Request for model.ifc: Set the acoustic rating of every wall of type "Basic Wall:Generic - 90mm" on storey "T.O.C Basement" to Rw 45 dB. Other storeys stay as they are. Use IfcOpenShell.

First a look at what the model holds.

```python
import ifcopenshell
import ifcopenshell.util.element

model = ifcopenshell.open("model.ifc")
print(model.schema)
storey = next(s for s in model.by_type("IfcBuildingStorey") if s.Name == "T.O.C Basement")
walls = [e for e in ifcopenshell.util.element.get_decomposition(storey) if e.is_a("IfcWall")]
seen = {}
for e in walls:
    element_type = ifcopenshell.util.element.get_type(e)
    key = (element_type.Name if element_type != e and element_type else None, ifcopenshell.util.element.get_pset(e, "Pset_WallCommon", "AcousticRating"))
    seen[key] = seen.get(key, 0) + 1
for (name, value), count in sorted(seen.items(), key=str):
    print(count, "x", name, "|", value)
```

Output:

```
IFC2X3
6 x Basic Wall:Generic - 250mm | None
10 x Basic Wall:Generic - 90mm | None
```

```python
import ifcopenshell
import ifcopenshell.api.pset
import ifcopenshell.util.element

model = ifcopenshell.open("model.ifc")

storey = next(s for s in model.by_type("IfcBuildingStorey") if s.Name == "T.O.C Basement")
walls = [e for e in ifcopenshell.util.element.get_decomposition(storey) if e.is_a("IfcWall")]

count = 0
for e in walls:
    element_type = ifcopenshell.util.element.get_type(e)
    if element_type in (None, e) or element_type.Name != "Basic Wall:Generic - 90mm":
        continue
    # add_pset returns the element's existing set when there is one.
    pset = ifcopenshell.api.pset.add_pset(model, product=e, name="Pset_WallCommon")
    ifcopenshell.api.pset.edit_pset(model, pset=pset, properties={"AcousticRating": "Rw 45 dB"})
    count += 1

print(count, "walls updated")

model.write("model-out.ifc")
```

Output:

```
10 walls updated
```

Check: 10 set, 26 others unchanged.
